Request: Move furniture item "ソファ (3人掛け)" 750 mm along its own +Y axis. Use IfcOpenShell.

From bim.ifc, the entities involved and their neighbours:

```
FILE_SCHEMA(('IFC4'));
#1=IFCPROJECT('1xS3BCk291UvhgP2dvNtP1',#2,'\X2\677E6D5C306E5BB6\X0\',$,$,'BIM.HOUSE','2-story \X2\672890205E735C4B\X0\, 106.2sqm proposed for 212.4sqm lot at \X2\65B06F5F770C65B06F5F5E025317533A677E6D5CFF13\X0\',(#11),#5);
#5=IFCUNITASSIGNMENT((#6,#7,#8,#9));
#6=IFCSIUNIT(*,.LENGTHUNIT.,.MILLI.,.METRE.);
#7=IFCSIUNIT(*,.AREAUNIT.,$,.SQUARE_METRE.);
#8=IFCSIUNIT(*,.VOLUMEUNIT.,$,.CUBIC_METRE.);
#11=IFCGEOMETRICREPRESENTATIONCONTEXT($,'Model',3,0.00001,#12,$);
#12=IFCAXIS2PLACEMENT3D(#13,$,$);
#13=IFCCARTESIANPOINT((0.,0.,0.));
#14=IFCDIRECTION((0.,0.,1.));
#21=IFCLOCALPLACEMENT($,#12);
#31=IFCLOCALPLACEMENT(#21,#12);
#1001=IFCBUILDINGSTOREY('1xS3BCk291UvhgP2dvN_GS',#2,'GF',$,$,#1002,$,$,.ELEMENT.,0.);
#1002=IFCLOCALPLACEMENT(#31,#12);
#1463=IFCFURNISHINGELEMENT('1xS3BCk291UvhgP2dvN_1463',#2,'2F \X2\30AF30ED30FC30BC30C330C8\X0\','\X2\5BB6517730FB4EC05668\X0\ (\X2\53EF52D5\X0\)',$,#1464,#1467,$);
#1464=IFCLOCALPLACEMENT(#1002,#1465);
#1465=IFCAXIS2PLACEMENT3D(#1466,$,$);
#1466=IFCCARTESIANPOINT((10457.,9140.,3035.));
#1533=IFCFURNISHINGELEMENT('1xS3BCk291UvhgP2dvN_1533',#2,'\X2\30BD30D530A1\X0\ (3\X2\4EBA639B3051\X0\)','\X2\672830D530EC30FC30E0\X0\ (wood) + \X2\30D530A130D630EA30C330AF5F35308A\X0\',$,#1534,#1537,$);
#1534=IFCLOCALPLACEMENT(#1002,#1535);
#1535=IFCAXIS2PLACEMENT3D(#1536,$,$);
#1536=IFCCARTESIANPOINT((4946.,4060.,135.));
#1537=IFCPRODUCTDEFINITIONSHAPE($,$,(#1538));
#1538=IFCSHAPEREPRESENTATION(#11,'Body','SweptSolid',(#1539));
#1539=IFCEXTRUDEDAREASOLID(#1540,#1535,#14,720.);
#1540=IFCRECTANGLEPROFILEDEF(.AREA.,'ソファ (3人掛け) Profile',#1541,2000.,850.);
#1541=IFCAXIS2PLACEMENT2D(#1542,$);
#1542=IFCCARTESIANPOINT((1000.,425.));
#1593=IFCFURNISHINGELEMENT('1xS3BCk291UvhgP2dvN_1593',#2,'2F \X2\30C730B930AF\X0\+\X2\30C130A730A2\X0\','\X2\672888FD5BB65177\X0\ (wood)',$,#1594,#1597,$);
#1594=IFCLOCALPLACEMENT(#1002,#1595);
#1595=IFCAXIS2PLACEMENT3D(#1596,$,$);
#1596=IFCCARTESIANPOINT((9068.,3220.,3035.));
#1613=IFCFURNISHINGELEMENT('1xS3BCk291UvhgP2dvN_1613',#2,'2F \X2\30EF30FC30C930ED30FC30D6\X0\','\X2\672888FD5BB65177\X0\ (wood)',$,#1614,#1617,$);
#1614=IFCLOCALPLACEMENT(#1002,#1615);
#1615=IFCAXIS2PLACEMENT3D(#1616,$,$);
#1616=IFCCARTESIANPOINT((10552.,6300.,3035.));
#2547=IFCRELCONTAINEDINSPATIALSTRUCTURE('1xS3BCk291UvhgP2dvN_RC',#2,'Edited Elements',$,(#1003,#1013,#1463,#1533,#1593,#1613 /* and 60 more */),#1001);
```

```python
import ifcopenshell
import ifcopenshell.api.geometry
import ifcopenshell.util.placement

model = ifcopenshell.open("bim.ifc")

item = model.by_id(1533)
matrix = ifcopenshell.util.placement.get_local_placement(item.ObjectPlacement)
matrix[:3, 3] += matrix[:3, 1] * 750.0
ifcopenshell.api.geometry.edit_object_placement(model, product=item, matrix=matrix, is_si=False)

print(ifcopenshell.util.placement.get_local_placement(item.ObjectPlacement).round(3) + 0.0)

model.write("bim_rev.ifc")
```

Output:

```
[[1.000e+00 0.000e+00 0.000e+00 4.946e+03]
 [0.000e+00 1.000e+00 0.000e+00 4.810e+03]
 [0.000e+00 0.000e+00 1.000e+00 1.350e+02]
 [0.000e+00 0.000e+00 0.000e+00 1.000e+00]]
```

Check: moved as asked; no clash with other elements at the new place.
